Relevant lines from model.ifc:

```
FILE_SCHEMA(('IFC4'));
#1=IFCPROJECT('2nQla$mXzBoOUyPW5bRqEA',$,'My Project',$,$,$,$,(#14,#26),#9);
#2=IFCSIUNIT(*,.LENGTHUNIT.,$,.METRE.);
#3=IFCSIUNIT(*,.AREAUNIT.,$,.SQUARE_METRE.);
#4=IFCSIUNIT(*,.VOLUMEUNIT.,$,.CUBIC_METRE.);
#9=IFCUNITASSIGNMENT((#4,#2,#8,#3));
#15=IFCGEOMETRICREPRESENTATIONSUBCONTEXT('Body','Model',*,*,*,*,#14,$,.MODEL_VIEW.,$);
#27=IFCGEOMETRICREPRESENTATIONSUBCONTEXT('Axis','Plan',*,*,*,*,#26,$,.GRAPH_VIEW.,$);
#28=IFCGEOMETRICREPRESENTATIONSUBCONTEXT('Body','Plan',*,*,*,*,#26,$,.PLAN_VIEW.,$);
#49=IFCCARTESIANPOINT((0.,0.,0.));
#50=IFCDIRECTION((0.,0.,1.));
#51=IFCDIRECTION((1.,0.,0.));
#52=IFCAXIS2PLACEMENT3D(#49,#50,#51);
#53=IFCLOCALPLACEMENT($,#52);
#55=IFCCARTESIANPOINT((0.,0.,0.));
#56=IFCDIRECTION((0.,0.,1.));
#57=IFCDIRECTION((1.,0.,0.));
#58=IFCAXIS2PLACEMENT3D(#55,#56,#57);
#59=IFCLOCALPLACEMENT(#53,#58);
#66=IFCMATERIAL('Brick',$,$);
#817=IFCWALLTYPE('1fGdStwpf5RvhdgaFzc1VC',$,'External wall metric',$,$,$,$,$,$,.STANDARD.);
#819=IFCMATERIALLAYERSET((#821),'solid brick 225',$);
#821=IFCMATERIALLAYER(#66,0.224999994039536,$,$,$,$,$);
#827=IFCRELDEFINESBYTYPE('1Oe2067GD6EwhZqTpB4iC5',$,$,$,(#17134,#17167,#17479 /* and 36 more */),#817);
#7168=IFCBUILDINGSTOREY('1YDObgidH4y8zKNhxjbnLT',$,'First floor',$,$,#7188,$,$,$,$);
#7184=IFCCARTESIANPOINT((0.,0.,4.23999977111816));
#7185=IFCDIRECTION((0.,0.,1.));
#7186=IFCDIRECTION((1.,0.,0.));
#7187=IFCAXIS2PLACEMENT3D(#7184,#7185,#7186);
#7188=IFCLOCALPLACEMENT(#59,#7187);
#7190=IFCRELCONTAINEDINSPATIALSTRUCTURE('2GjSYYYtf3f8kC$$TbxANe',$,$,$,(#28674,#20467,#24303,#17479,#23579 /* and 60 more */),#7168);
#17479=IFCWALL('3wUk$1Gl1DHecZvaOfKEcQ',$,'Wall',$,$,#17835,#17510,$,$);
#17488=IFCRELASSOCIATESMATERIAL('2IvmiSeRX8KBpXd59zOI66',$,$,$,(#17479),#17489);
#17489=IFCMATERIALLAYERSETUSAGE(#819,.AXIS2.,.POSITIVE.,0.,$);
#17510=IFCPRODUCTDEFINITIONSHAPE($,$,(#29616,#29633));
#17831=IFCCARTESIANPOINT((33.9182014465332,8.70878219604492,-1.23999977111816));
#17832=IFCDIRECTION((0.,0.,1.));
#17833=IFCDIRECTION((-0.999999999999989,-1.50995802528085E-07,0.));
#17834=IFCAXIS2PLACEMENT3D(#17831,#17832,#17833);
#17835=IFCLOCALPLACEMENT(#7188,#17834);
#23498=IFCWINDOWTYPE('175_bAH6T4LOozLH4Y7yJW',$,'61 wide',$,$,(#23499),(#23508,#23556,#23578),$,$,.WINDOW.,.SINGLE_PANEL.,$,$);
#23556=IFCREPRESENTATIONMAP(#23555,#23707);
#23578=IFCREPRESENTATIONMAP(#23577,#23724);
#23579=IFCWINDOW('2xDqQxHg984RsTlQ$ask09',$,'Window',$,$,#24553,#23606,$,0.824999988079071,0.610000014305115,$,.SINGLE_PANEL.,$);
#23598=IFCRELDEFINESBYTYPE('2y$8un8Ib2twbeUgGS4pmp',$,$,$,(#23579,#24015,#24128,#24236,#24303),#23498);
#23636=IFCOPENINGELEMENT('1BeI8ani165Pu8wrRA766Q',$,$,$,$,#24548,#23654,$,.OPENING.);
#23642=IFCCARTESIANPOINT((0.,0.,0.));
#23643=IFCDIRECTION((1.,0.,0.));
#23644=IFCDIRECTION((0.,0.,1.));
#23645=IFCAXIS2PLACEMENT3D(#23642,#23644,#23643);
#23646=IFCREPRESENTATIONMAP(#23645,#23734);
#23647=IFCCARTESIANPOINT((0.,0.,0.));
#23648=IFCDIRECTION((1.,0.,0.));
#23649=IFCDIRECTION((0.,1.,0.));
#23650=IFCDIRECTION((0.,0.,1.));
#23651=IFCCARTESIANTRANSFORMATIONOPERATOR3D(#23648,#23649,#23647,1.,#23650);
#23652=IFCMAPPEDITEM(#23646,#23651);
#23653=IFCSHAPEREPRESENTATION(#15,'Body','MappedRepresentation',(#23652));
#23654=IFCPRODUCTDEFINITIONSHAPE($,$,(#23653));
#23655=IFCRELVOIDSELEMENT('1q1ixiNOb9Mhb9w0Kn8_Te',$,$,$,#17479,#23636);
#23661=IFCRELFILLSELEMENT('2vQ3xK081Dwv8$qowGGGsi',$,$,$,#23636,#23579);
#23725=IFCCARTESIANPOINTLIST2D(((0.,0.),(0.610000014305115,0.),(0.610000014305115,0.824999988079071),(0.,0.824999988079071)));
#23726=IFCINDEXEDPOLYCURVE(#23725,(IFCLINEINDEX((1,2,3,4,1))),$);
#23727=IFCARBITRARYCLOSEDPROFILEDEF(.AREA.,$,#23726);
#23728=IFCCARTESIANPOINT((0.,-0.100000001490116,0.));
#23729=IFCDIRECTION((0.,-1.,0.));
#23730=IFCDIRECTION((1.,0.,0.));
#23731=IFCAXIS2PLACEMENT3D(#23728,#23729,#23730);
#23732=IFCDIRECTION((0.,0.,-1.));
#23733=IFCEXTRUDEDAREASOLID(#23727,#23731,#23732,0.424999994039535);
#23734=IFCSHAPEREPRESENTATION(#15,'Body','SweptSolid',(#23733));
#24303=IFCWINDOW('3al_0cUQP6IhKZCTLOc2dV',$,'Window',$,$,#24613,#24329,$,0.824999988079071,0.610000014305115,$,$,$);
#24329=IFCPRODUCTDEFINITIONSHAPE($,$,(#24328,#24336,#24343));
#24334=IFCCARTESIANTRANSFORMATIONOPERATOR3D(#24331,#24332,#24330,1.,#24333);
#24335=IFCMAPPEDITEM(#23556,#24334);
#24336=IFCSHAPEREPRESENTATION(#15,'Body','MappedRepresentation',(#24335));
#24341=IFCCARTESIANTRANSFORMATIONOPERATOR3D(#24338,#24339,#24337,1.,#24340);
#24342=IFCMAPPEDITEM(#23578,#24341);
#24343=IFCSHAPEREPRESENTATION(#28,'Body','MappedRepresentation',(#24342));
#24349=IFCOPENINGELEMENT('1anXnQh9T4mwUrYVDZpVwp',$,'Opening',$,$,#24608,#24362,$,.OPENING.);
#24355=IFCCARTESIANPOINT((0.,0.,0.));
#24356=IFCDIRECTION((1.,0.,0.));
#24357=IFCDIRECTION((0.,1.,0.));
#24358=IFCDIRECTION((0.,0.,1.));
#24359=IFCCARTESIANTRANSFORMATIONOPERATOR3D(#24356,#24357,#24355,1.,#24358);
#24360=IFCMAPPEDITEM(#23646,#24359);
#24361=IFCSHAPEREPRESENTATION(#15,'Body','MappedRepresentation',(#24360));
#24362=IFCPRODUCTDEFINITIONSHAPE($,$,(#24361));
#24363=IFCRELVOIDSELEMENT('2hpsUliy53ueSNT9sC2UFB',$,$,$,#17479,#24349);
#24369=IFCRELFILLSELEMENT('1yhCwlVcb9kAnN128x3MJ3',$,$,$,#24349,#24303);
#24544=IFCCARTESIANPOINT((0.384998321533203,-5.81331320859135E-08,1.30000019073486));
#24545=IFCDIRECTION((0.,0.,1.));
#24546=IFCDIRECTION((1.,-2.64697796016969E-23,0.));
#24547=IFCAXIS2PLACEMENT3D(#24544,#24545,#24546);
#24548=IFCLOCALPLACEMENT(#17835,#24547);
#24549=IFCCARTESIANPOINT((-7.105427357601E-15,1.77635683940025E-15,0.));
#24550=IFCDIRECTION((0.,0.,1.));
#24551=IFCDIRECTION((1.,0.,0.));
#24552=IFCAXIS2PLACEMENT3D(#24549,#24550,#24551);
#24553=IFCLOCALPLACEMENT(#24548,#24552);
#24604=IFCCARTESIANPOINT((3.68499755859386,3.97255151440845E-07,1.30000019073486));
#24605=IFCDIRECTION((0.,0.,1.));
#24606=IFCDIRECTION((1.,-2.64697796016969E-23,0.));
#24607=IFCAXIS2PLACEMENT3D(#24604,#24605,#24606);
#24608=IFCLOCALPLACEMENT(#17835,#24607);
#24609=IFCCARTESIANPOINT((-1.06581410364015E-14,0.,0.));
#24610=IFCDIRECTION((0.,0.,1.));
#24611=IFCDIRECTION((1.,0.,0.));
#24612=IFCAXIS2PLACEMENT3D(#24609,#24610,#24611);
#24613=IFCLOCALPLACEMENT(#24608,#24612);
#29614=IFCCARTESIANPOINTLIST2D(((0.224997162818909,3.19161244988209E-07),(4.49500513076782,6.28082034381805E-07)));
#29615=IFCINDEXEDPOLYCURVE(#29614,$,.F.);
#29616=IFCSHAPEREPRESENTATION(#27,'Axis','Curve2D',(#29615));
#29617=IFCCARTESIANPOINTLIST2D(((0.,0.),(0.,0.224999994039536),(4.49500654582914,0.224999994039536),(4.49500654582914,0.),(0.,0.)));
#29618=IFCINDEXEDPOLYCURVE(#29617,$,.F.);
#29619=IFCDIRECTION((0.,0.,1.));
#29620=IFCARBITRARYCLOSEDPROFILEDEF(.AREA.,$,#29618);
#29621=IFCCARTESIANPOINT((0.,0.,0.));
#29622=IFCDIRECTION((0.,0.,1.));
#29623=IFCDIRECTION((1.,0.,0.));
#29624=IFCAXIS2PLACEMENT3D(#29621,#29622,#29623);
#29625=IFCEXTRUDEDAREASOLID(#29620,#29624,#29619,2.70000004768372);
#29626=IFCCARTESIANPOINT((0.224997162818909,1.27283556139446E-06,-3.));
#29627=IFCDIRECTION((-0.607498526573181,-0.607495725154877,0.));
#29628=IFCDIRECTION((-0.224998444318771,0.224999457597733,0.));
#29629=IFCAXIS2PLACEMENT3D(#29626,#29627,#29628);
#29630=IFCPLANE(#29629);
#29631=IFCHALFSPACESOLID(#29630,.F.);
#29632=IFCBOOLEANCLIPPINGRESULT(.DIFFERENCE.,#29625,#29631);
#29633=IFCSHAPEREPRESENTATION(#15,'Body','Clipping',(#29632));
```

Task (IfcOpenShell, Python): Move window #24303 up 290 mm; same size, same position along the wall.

```python
import numpy as np
import ifcopenshell
import ifcopenshell.api.geometry
import ifcopenshell.util.placement
import ifcopenshell.util.unit

model = ifcopenshell.open("model.ifc")
unit_scale = ifcopenshell.util.unit.calculate_unit_scale(model)

window = model.by_guid("3al_0cUQP6IhKZCTLOc2dV")
opening = window.FillsVoids[0].RelatingOpeningElement
dz = 0.29

shift = np.array([0.0, 0.0, dz])
# The window is placed relative to its opening, so it follows when the opening moves.
matrix = ifcopenshell.util.placement.get_local_placement(opening.ObjectPlacement)
matrix[:3, 3] += shift
ifcopenshell.api.geometry.edit_object_placement(
    model, product=opening, matrix=matrix, is_si=False, should_transform_children=True
)

print(f"moved by {dz * unit_scale:+.3f} m")

model.write("model_updated.ifc")
```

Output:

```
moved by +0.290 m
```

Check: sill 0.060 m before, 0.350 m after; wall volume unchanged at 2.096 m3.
